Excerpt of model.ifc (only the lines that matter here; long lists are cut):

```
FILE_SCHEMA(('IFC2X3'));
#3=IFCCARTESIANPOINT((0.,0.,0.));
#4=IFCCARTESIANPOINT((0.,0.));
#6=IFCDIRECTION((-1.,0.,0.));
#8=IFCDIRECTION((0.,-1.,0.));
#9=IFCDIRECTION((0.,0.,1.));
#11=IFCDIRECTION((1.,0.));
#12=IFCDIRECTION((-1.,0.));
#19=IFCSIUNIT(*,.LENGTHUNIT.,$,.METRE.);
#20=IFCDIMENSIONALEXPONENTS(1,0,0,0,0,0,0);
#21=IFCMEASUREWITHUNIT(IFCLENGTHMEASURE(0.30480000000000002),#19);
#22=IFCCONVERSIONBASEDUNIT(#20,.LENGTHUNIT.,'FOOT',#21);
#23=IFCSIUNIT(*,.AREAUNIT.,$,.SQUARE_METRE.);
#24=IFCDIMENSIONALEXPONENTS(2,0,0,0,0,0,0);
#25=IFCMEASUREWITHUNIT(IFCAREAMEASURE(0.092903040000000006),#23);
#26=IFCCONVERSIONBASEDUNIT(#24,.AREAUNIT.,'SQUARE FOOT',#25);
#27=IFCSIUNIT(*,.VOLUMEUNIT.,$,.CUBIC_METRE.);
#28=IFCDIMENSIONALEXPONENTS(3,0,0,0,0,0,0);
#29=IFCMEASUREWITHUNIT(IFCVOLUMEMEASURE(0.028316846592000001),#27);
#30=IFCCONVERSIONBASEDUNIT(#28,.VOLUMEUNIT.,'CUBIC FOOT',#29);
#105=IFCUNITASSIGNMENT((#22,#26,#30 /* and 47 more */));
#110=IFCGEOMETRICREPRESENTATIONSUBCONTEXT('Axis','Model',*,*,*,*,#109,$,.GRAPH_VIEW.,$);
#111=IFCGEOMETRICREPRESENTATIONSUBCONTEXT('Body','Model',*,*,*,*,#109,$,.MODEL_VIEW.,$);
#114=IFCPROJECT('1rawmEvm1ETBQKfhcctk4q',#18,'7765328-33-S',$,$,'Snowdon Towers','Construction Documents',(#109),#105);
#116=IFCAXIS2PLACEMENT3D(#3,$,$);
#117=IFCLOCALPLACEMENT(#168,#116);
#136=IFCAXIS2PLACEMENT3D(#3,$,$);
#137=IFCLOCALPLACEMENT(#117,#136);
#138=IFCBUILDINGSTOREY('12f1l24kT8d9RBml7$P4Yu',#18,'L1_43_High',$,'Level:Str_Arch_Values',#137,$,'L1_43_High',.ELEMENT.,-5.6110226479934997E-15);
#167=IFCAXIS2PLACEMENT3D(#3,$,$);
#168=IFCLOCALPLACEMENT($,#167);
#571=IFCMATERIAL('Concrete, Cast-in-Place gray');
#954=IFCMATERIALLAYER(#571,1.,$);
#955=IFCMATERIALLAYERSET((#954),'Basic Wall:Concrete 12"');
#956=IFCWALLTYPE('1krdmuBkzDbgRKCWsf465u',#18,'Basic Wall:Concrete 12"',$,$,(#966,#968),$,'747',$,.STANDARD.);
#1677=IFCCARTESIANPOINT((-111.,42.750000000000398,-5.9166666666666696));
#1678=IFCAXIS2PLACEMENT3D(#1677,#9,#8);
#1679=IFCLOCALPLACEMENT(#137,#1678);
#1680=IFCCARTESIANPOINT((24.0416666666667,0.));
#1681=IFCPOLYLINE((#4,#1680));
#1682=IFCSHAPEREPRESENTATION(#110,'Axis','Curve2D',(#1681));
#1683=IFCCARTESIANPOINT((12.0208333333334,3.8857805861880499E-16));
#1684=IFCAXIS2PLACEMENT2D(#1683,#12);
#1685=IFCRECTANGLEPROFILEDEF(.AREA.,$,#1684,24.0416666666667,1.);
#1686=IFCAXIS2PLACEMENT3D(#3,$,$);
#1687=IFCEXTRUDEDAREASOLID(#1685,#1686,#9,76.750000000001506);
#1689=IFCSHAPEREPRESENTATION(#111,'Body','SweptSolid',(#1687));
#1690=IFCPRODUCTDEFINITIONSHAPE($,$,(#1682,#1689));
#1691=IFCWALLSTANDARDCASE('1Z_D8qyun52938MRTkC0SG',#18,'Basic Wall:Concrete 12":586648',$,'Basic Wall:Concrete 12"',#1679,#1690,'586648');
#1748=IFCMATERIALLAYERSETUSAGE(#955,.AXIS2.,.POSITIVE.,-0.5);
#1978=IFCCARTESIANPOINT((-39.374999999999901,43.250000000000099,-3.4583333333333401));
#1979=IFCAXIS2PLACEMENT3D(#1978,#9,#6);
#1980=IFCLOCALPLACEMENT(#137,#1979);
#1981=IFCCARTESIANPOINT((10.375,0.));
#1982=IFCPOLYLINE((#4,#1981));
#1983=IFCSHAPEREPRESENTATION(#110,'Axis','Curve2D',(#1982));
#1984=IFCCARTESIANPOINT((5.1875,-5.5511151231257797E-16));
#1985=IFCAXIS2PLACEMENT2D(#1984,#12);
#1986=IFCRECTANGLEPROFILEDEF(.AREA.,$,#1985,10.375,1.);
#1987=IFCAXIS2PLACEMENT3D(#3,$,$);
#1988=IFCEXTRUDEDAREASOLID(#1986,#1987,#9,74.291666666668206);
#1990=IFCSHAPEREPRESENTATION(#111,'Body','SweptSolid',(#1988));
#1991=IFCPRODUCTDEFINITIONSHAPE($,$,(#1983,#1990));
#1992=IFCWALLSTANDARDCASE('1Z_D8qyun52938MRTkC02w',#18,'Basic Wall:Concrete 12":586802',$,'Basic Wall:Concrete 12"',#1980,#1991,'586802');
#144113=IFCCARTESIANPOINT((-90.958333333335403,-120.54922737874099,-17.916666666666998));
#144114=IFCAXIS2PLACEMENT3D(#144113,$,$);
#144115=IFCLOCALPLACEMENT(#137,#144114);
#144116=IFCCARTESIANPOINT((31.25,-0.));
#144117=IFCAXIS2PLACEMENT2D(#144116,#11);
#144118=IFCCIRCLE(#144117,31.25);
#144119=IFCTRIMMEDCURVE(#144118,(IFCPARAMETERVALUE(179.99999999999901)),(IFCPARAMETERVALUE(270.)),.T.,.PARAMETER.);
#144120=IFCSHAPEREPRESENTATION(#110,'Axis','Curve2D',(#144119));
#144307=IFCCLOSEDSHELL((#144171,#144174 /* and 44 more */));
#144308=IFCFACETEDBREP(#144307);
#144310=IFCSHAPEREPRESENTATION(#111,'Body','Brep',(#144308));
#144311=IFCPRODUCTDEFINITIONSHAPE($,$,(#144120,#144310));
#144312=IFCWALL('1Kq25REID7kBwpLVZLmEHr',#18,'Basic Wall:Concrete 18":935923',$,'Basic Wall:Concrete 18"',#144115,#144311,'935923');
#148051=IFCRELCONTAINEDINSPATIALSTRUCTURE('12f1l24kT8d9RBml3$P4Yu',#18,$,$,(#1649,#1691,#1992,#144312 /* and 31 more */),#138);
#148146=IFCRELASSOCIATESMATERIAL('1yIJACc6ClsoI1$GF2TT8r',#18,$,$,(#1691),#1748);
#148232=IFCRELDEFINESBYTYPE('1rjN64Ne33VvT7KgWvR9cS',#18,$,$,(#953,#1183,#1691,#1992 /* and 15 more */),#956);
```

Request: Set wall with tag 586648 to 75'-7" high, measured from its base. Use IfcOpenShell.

```python
import ifcopenshell
import ifcopenshell.geom
import ifcopenshell.util.representation
import ifcopenshell.util.shape
import ifcopenshell.util.unit

model = ifcopenshell.open("model.ifc")
unit_scale = ifcopenshell.util.unit.calculate_unit_scale(model)
settings = ifcopenshell.geom.settings()


def volume(element):
    """Net volume in cubic metres, openings subtracted."""
    shape = ifcopenshell.geom.create_shape(settings, element)
    return ifcopenshell.util.shape.get_volume(shape.geometry)


wall = model.by_id(1691)
before = volume(wall)

body = ifcopenshell.util.representation.get_representation(wall, "Model", "Body")
solid = body.Items[0]
old_height = solid.Depth
solid.Depth = 907 * 0.0254 / unit_scale
after = volume(wall)

print(f"height {old_height:g} -> {solid.Depth:g}, volume {before:.3f} -> {after:.3f} m3")

model.write("model_updated.ifc")
```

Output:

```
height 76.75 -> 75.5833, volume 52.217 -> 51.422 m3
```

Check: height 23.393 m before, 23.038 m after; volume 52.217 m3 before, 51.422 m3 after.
